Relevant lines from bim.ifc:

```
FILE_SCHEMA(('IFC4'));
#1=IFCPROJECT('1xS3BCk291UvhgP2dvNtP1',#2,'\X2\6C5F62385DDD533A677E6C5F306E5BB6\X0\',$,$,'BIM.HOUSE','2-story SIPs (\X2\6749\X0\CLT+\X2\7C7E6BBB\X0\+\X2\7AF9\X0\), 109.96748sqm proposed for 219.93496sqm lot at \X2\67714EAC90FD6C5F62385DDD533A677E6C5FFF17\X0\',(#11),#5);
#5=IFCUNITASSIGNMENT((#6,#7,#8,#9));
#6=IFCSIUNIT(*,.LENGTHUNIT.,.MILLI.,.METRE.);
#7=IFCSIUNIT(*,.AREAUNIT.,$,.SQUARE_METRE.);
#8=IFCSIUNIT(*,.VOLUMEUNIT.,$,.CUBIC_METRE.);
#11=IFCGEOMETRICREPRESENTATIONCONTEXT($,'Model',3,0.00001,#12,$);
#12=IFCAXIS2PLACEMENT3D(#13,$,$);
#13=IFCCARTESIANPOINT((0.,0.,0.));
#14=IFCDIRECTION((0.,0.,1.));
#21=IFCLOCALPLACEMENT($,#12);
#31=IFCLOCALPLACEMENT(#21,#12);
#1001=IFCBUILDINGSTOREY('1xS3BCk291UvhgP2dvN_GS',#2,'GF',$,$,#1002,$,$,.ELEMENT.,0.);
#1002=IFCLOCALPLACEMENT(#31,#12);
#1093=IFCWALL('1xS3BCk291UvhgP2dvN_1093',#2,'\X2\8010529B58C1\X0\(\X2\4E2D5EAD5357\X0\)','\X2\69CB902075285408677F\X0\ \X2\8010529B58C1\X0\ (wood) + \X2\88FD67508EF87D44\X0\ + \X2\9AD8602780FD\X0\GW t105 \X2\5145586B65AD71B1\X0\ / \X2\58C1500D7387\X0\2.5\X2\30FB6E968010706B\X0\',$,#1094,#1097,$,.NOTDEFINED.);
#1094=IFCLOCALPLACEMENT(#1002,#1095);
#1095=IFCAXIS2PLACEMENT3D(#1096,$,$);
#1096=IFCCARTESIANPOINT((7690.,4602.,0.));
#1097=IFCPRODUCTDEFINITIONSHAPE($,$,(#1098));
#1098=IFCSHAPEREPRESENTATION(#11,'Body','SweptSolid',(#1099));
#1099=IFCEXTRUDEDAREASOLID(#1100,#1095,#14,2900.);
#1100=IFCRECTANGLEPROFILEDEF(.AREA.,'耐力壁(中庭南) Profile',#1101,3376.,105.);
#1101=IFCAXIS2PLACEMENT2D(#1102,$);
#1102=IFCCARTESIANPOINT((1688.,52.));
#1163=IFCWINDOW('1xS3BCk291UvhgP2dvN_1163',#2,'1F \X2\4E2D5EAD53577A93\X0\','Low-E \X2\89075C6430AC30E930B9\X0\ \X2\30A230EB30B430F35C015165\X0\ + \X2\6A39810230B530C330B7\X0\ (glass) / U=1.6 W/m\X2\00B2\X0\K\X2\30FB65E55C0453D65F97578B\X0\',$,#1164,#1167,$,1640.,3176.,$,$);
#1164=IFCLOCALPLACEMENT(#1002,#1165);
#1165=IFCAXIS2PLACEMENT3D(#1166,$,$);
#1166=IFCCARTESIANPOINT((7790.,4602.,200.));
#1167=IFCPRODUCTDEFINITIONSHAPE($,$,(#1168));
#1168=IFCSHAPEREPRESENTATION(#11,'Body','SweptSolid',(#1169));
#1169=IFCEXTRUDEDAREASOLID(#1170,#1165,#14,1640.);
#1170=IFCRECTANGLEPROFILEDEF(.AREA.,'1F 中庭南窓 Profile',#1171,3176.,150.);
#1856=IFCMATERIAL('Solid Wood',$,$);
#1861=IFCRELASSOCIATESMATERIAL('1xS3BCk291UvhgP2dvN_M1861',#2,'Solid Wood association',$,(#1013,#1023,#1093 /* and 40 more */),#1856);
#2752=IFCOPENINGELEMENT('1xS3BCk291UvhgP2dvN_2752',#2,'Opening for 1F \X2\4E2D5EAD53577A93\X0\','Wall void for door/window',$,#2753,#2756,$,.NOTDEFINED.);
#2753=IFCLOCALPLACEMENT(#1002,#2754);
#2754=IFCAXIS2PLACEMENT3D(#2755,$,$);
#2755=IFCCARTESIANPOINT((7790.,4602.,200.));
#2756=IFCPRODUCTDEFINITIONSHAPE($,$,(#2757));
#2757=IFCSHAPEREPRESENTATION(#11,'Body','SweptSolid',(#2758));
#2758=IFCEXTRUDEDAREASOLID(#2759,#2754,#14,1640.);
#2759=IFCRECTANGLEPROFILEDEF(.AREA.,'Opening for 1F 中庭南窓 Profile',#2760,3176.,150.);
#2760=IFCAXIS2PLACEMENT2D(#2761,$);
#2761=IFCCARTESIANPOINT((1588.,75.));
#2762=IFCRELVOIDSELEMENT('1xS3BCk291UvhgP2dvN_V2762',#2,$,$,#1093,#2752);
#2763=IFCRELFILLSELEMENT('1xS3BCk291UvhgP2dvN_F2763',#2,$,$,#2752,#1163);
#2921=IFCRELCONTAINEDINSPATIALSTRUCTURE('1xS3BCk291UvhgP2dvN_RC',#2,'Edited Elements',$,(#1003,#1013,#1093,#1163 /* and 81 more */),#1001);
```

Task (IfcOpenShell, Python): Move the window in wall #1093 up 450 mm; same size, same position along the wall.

```python
import numpy as np
import ifcopenshell
import ifcopenshell.api.geometry
import ifcopenshell.util.placement
import ifcopenshell.util.unit

model = ifcopenshell.open("bim.ifc")
unit_scale = ifcopenshell.util.unit.calculate_unit_scale(model)

window = model.by_guid("1xS3BCk291UvhgP2dvN_1163")
opening = window.FillsVoids[0].RelatingOpeningElement
dz = 0.45 / unit_scale

shift = np.array([0.0, 0.0, dz])
# The window is not placed relative to its opening, so move both.
for product in (opening, window):
    matrix = ifcopenshell.util.placement.get_local_placement(product.ObjectPlacement)
    matrix[:3, 3] += shift
    ifcopenshell.api.geometry.edit_object_placement(model, product=product, matrix=matrix, is_si=False)

print(f"moved by {dz * unit_scale:+.3f} m")

model.write("bim_edited.ifc")
```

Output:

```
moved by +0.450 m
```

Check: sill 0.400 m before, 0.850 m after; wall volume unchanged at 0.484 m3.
